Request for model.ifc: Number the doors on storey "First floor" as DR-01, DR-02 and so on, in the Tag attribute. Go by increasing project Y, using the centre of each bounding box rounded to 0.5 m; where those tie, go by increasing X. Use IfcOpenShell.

First a look at what the model holds.

```python
import ifcopenshell
import ifcopenshell.util.element
import ifcopenshell.util.placement

model = ifcopenshell.open("model.ifc")
print(model.schema)
storey = next(s for s in model.by_type("IfcBuildingStorey") if s.Name == "First floor")
doors = [e for e in ifcopenshell.util.element.get_decomposition(storey) if e.is_a("IfcDoor")]
for e in sorted(doors, key=lambda e: e.id()):
    origin = ifcopenshell.util.placement.get_local_placement(e.ObjectPlacement)[:3, 3]
    print(e.id(), e.Tag, e.Name, origin.round(2) + 0.0, sep=" | ")
```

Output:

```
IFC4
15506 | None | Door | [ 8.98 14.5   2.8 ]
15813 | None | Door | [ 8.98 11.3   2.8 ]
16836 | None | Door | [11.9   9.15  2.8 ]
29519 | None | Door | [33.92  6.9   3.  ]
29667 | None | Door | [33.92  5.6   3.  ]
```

```python
import ifcopenshell
import ifcopenshell.geom
import ifcopenshell.util.element
import ifcopenshell.util.shape

model = ifcopenshell.open("model.ifc")
settings = ifcopenshell.geom.settings()
settings.set("use-world-coords", True)


def centre(element):
    shape = ifcopenshell.geom.create_shape(settings, element)
    return ifcopenshell.util.shape.get_bbox_centroid(shape.geometry)


storey = next(s for s in model.by_type("IfcBuildingStorey") if s.Name == "First floor")
doors = [e for e in ifcopenshell.util.element.get_decomposition(storey) if e.is_a("IfcDoor")]

# Insertion points can sit at a corner or the storey origin, so sort by the geometry (in metres).
centres = {e: centre(e) for e in doors}
doors.sort(key=lambda e: (round(centres[e][1] / 0.5), centres[e][0]))

for i, e in enumerate(doors, start=1):
    number = f"DR-{i:02d}"
    e.Tag = number
    print(e.id(), number)

model.write("model_updated.ifc")
```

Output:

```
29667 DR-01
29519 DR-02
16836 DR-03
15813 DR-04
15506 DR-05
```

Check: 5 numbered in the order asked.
